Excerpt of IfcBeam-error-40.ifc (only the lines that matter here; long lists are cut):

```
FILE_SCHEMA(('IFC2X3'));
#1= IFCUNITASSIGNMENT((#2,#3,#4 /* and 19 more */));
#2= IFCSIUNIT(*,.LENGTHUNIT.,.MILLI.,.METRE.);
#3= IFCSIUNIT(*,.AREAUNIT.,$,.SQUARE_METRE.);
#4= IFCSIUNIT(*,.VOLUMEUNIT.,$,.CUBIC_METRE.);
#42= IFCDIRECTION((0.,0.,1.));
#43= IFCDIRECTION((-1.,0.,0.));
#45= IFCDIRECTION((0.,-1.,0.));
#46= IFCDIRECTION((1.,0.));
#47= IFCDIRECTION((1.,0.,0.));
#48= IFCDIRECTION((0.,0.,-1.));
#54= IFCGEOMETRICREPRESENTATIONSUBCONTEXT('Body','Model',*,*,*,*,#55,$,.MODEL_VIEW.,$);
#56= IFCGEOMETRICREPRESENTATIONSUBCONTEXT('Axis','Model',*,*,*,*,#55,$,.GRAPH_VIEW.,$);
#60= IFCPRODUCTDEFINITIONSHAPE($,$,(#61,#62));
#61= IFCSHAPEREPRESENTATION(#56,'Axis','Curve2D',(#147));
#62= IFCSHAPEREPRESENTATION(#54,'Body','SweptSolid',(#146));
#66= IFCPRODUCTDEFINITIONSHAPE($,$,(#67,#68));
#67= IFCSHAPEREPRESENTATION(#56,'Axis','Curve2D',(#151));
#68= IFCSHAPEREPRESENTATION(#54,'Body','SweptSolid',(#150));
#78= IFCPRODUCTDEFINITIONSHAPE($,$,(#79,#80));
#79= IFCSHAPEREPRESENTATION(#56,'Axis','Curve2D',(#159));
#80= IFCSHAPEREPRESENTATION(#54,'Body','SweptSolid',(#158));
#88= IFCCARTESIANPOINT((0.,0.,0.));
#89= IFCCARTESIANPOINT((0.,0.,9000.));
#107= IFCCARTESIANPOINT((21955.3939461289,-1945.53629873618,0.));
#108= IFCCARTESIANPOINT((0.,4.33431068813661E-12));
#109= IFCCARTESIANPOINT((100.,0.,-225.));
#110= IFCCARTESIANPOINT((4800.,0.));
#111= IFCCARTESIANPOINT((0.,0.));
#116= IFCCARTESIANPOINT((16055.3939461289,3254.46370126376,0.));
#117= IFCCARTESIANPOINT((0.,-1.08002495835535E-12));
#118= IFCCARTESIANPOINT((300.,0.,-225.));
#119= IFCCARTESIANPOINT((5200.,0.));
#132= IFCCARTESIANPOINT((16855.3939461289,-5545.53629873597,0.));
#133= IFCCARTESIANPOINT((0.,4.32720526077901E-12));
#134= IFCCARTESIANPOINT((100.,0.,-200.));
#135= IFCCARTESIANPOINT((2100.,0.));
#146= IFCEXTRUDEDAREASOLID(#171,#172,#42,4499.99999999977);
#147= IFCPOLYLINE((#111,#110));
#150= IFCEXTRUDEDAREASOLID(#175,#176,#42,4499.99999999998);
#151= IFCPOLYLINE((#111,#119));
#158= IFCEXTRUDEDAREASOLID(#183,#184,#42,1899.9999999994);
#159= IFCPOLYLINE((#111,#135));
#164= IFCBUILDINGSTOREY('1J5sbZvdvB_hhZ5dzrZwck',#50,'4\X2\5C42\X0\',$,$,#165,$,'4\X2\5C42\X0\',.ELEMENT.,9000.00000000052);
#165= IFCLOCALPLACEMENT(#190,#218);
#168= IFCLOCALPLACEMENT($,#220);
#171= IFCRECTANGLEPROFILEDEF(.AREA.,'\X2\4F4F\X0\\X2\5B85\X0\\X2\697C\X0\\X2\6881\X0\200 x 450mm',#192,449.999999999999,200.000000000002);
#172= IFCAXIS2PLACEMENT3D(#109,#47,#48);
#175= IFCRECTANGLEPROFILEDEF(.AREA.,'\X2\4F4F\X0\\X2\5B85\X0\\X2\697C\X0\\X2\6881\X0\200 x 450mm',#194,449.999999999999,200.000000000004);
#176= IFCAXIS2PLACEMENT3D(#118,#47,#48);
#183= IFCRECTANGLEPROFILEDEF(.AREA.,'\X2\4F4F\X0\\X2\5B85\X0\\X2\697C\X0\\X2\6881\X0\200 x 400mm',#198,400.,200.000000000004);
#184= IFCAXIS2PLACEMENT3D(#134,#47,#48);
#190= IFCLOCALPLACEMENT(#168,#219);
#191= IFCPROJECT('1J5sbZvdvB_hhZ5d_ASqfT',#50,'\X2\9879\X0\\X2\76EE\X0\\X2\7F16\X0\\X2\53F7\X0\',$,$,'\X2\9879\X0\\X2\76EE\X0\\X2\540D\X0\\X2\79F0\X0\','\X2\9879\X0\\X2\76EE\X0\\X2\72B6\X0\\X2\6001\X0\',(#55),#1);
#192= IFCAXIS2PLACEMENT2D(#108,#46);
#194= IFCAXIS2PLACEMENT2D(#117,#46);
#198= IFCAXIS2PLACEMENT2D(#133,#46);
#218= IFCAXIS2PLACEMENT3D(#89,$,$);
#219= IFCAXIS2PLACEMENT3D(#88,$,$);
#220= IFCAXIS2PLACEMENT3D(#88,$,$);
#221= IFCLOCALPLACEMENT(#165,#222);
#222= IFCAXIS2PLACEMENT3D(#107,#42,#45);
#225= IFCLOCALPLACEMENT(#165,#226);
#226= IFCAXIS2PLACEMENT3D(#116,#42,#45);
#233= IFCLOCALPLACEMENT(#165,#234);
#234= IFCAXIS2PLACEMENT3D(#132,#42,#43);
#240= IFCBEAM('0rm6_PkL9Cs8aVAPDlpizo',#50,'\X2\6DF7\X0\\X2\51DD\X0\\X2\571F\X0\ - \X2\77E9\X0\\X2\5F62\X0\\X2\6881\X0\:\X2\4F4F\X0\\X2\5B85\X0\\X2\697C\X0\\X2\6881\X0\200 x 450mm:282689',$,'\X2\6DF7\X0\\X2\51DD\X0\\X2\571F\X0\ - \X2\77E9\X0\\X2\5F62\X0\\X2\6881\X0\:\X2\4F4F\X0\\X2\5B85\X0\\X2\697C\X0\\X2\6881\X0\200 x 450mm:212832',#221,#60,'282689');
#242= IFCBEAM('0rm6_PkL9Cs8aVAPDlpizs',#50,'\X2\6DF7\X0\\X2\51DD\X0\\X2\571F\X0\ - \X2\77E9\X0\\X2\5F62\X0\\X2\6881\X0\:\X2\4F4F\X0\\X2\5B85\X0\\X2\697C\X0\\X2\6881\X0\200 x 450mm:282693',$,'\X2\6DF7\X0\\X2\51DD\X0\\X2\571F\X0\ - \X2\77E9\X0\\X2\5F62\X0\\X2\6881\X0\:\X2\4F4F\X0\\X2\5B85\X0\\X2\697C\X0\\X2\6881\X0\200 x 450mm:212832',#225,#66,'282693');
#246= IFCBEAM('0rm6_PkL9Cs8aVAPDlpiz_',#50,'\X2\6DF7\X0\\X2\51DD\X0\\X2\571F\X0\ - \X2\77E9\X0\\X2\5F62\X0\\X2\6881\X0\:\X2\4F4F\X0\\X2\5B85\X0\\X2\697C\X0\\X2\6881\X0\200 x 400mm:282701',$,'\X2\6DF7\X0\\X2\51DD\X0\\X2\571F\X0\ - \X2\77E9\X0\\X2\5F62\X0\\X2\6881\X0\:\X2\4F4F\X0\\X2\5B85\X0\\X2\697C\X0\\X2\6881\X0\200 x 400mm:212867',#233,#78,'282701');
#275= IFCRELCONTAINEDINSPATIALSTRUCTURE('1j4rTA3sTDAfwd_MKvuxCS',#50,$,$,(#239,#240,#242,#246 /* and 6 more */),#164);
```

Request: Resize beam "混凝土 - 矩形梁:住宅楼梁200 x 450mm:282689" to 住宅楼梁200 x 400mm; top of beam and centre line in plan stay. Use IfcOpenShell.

```python
import ifcopenshell
import ifcopenshell.util.element
import ifcopenshell.util.representation

model = ifcopenshell.open("IfcBeam-error-40.ifc")

member = model.by_guid("0rm6_PkL9Cs8aVAPDlpizo")
source = next(p for p in model.by_type("IfcRectangleProfileDef") if p.ProfileName == "住宅楼梁200 x 400mm")

body = ifcopenshell.util.representation.get_representation(member, "Model", "Body")
solid = body.Items[0]
old_profile = solid.SweptArea

# Copy the section's sizes but keep this member's own profile position.
profile = ifcopenshell.util.element.copy(model, source)
# Profiles are centred, so shift by half the change in depth to hold the top.
shift = (old_profile.XDim - profile.XDim) / 2
x, y = old_profile.Position.Location.Coordinates
up = (-1.0, 0.0)  # upwards, in the solid's own plane
location = model.createIfcCartesianPoint((x + up[0] * shift, y + up[1] * shift))
profile.Position = model.createIfcAxis2Placement2D(location, old_profile.Position.RefDirection)
solid.SweptArea = profile
if not model.get_total_inverses(old_profile):
    ifcopenshell.util.element.remove_deep2(model, old_profile)
member.Name = member.Name.replace("住宅楼梁200 x 450mm", "住宅楼梁200 x 400mm")
member.ObjectType = member.ObjectType.replace("住宅楼梁200 x 450mm", "住宅楼梁200 x 400mm")

print(solid.SweptArea)

model.write("IfcBeam-error-40_updated.ifc")
```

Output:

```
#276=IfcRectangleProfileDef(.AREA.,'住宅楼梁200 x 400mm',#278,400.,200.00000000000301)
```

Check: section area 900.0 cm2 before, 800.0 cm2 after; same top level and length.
